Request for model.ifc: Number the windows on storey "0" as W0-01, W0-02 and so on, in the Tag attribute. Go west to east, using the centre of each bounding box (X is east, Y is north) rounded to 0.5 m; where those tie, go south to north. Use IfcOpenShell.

First a look at what the model holds.

```python
import ifcopenshell
import ifcopenshell.util.element
import ifcopenshell.util.placement

model = ifcopenshell.open("model.ifc")
print(model.schema)
storey = next(s for s in model.by_type("IfcBuildingStorey") if s.Name == "0")
windows = [e for e in ifcopenshell.util.element.get_decomposition(storey) if e.is_a("IfcWindow")]
for e in sorted(windows, key=lambda e: e.id()):
    origin = ifcopenshell.util.placement.get_local_placement(e.ObjectPlacement)[:3, 3]
    print(e.id(), e.Tag, e.Name, origin.round(2) + 0.0, sep=" | ")
```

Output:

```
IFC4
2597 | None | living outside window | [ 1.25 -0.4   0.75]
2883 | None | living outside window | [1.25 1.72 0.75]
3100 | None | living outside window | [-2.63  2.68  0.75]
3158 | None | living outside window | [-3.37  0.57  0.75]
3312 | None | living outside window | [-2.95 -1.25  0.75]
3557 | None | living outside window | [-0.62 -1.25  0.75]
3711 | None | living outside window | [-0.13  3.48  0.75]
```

```python
import ifcopenshell
import ifcopenshell.geom
import ifcopenshell.util.element
import ifcopenshell.util.shape

model = ifcopenshell.open("model.ifc")
settings = ifcopenshell.geom.settings()
settings.set("use-world-coords", True)


def centre(element):
    shape = ifcopenshell.geom.create_shape(settings, element)
    return ifcopenshell.util.shape.get_bbox_centroid(shape.geometry)


storey = next(s for s in model.by_type("IfcBuildingStorey") if s.Name == "0")
windows = [e for e in ifcopenshell.util.element.get_decomposition(storey) if e.is_a("IfcWindow")]

# Insertion points can sit at a corner or the storey origin, so sort by the geometry (in metres).
centres = {e: centre(e) for e in windows}
windows.sort(key=lambda e: (round(centres[e][0] / 0.5), centres[e][1]))

for i, e in enumerate(windows, start=1):
    number = f"W0-{i:02d}"
    e.Tag = number
    print(e.id(), number)

model.write("model_updated.ifc")
```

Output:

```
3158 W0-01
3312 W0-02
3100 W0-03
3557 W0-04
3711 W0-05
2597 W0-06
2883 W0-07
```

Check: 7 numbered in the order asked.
